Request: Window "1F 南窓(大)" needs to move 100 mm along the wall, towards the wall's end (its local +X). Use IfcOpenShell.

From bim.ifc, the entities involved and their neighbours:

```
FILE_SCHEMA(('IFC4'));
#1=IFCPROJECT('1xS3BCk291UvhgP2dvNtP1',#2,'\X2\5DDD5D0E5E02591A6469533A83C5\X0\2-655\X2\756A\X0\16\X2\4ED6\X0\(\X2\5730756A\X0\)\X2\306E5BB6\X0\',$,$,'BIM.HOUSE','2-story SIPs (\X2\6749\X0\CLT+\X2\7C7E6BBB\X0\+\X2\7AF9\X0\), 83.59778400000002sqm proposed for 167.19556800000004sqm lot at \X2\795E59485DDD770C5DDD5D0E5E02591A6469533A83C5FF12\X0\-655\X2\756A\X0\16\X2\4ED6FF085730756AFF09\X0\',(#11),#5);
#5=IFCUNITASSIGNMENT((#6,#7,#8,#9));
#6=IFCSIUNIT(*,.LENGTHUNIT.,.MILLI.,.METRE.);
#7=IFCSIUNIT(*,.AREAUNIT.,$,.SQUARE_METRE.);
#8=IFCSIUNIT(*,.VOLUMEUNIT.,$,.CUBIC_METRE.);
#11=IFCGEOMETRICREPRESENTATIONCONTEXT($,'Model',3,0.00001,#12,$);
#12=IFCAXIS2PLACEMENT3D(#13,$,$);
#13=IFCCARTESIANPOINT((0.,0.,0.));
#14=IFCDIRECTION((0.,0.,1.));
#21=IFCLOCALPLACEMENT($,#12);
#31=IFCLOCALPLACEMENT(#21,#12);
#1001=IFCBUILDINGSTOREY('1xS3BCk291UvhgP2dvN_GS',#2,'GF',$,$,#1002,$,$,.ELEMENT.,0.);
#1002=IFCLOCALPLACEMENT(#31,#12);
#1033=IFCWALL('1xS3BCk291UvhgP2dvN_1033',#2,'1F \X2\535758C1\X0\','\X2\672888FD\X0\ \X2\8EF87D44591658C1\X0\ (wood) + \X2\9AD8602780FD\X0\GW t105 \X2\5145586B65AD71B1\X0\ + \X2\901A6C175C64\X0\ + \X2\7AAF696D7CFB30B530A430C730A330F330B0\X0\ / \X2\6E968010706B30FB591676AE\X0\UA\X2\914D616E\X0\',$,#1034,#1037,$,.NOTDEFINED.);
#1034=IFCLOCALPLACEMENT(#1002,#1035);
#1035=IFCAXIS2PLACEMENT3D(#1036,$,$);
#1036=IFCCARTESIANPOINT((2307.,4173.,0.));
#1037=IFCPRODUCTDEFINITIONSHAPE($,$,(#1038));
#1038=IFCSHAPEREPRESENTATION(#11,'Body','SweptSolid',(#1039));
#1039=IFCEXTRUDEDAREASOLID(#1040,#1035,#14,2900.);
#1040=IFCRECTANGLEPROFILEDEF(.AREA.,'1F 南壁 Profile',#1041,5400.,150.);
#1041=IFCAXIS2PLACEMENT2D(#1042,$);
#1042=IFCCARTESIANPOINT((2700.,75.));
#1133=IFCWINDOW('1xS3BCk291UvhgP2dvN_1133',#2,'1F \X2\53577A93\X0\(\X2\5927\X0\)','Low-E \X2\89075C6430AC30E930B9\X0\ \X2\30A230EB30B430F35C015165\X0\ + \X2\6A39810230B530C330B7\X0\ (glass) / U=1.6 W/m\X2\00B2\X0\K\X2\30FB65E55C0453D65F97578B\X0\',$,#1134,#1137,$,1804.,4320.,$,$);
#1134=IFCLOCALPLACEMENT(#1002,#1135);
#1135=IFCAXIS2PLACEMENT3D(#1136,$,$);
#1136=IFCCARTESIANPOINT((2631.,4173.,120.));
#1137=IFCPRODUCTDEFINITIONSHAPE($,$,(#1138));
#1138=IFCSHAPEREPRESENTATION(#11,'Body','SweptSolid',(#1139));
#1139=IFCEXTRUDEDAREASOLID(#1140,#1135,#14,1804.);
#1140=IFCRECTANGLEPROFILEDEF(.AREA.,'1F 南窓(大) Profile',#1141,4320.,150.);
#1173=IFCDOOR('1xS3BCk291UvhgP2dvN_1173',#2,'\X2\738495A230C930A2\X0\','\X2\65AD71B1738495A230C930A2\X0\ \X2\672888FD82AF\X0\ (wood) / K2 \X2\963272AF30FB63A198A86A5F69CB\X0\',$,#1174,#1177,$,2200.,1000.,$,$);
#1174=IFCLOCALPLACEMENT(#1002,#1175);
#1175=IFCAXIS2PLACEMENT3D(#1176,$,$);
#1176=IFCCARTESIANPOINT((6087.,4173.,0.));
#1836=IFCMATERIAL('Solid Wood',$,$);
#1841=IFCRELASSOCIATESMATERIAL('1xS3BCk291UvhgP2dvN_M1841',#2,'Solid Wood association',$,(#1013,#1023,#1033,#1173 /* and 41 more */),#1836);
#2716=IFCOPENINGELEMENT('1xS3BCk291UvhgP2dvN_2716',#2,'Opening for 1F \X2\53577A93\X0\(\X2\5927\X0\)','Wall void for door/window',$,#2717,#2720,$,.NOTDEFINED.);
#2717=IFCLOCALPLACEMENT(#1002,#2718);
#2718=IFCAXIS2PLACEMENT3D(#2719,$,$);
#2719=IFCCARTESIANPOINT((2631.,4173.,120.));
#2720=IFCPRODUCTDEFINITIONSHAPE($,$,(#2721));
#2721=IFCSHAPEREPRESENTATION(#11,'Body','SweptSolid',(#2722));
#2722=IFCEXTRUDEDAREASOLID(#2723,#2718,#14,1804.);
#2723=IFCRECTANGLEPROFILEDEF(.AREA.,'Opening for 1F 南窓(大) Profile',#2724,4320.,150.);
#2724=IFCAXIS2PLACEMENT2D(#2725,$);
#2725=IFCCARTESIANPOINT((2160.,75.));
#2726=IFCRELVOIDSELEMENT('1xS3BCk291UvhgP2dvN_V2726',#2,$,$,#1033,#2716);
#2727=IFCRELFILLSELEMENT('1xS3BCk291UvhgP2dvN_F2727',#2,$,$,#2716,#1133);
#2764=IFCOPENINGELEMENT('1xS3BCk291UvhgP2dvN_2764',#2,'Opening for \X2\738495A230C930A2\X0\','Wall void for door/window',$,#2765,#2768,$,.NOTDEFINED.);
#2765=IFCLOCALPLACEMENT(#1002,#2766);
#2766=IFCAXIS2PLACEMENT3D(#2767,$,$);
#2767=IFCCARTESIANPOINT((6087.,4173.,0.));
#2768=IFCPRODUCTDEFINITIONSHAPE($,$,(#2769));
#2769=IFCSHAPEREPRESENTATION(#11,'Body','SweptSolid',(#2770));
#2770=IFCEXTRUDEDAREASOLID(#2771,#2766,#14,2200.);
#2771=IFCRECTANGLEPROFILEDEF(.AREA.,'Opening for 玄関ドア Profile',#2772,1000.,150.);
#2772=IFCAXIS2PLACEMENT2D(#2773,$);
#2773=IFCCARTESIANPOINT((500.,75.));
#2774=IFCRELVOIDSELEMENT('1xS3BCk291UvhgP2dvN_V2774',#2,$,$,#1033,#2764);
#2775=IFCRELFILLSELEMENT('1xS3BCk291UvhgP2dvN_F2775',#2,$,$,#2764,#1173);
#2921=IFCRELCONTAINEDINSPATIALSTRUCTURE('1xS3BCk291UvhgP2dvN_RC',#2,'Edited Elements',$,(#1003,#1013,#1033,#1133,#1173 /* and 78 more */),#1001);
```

```python
import ifcopenshell
import ifcopenshell.api.geometry
import ifcopenshell.util.placement
import ifcopenshell.util.unit

model = ifcopenshell.open("bim.ifc")
unit_scale = ifcopenshell.util.unit.calculate_unit_scale(model)

window = model.by_id(1133)
opening = window.FillsVoids[0].RelatingOpeningElement
wall = opening.VoidsElements[0].RelatingBuildingElement

wall_matrix = ifcopenshell.util.placement.get_local_placement(wall.ObjectPlacement)
shift = wall_matrix[:3, 0] * 0.1 / unit_scale
before = ifcopenshell.util.placement.get_local_placement(window.ObjectPlacement)[:3, 3].copy()

# The window is not placed relative to its opening, so move both.
for product in (opening, window):
    matrix = ifcopenshell.util.placement.get_local_placement(product.ObjectPlacement)
    matrix[:3, 3] += shift
    ifcopenshell.api.geometry.edit_object_placement(model, product=product, matrix=matrix, is_si=False)

after = ifcopenshell.util.placement.get_local_placement(window.ObjectPlacement)[:3, 3]
print("window moved by", (after - before).round(3) + 0.0)

model.write("bim_v2.ifc")
```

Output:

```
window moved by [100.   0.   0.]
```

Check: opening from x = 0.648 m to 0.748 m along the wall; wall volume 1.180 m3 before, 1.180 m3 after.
